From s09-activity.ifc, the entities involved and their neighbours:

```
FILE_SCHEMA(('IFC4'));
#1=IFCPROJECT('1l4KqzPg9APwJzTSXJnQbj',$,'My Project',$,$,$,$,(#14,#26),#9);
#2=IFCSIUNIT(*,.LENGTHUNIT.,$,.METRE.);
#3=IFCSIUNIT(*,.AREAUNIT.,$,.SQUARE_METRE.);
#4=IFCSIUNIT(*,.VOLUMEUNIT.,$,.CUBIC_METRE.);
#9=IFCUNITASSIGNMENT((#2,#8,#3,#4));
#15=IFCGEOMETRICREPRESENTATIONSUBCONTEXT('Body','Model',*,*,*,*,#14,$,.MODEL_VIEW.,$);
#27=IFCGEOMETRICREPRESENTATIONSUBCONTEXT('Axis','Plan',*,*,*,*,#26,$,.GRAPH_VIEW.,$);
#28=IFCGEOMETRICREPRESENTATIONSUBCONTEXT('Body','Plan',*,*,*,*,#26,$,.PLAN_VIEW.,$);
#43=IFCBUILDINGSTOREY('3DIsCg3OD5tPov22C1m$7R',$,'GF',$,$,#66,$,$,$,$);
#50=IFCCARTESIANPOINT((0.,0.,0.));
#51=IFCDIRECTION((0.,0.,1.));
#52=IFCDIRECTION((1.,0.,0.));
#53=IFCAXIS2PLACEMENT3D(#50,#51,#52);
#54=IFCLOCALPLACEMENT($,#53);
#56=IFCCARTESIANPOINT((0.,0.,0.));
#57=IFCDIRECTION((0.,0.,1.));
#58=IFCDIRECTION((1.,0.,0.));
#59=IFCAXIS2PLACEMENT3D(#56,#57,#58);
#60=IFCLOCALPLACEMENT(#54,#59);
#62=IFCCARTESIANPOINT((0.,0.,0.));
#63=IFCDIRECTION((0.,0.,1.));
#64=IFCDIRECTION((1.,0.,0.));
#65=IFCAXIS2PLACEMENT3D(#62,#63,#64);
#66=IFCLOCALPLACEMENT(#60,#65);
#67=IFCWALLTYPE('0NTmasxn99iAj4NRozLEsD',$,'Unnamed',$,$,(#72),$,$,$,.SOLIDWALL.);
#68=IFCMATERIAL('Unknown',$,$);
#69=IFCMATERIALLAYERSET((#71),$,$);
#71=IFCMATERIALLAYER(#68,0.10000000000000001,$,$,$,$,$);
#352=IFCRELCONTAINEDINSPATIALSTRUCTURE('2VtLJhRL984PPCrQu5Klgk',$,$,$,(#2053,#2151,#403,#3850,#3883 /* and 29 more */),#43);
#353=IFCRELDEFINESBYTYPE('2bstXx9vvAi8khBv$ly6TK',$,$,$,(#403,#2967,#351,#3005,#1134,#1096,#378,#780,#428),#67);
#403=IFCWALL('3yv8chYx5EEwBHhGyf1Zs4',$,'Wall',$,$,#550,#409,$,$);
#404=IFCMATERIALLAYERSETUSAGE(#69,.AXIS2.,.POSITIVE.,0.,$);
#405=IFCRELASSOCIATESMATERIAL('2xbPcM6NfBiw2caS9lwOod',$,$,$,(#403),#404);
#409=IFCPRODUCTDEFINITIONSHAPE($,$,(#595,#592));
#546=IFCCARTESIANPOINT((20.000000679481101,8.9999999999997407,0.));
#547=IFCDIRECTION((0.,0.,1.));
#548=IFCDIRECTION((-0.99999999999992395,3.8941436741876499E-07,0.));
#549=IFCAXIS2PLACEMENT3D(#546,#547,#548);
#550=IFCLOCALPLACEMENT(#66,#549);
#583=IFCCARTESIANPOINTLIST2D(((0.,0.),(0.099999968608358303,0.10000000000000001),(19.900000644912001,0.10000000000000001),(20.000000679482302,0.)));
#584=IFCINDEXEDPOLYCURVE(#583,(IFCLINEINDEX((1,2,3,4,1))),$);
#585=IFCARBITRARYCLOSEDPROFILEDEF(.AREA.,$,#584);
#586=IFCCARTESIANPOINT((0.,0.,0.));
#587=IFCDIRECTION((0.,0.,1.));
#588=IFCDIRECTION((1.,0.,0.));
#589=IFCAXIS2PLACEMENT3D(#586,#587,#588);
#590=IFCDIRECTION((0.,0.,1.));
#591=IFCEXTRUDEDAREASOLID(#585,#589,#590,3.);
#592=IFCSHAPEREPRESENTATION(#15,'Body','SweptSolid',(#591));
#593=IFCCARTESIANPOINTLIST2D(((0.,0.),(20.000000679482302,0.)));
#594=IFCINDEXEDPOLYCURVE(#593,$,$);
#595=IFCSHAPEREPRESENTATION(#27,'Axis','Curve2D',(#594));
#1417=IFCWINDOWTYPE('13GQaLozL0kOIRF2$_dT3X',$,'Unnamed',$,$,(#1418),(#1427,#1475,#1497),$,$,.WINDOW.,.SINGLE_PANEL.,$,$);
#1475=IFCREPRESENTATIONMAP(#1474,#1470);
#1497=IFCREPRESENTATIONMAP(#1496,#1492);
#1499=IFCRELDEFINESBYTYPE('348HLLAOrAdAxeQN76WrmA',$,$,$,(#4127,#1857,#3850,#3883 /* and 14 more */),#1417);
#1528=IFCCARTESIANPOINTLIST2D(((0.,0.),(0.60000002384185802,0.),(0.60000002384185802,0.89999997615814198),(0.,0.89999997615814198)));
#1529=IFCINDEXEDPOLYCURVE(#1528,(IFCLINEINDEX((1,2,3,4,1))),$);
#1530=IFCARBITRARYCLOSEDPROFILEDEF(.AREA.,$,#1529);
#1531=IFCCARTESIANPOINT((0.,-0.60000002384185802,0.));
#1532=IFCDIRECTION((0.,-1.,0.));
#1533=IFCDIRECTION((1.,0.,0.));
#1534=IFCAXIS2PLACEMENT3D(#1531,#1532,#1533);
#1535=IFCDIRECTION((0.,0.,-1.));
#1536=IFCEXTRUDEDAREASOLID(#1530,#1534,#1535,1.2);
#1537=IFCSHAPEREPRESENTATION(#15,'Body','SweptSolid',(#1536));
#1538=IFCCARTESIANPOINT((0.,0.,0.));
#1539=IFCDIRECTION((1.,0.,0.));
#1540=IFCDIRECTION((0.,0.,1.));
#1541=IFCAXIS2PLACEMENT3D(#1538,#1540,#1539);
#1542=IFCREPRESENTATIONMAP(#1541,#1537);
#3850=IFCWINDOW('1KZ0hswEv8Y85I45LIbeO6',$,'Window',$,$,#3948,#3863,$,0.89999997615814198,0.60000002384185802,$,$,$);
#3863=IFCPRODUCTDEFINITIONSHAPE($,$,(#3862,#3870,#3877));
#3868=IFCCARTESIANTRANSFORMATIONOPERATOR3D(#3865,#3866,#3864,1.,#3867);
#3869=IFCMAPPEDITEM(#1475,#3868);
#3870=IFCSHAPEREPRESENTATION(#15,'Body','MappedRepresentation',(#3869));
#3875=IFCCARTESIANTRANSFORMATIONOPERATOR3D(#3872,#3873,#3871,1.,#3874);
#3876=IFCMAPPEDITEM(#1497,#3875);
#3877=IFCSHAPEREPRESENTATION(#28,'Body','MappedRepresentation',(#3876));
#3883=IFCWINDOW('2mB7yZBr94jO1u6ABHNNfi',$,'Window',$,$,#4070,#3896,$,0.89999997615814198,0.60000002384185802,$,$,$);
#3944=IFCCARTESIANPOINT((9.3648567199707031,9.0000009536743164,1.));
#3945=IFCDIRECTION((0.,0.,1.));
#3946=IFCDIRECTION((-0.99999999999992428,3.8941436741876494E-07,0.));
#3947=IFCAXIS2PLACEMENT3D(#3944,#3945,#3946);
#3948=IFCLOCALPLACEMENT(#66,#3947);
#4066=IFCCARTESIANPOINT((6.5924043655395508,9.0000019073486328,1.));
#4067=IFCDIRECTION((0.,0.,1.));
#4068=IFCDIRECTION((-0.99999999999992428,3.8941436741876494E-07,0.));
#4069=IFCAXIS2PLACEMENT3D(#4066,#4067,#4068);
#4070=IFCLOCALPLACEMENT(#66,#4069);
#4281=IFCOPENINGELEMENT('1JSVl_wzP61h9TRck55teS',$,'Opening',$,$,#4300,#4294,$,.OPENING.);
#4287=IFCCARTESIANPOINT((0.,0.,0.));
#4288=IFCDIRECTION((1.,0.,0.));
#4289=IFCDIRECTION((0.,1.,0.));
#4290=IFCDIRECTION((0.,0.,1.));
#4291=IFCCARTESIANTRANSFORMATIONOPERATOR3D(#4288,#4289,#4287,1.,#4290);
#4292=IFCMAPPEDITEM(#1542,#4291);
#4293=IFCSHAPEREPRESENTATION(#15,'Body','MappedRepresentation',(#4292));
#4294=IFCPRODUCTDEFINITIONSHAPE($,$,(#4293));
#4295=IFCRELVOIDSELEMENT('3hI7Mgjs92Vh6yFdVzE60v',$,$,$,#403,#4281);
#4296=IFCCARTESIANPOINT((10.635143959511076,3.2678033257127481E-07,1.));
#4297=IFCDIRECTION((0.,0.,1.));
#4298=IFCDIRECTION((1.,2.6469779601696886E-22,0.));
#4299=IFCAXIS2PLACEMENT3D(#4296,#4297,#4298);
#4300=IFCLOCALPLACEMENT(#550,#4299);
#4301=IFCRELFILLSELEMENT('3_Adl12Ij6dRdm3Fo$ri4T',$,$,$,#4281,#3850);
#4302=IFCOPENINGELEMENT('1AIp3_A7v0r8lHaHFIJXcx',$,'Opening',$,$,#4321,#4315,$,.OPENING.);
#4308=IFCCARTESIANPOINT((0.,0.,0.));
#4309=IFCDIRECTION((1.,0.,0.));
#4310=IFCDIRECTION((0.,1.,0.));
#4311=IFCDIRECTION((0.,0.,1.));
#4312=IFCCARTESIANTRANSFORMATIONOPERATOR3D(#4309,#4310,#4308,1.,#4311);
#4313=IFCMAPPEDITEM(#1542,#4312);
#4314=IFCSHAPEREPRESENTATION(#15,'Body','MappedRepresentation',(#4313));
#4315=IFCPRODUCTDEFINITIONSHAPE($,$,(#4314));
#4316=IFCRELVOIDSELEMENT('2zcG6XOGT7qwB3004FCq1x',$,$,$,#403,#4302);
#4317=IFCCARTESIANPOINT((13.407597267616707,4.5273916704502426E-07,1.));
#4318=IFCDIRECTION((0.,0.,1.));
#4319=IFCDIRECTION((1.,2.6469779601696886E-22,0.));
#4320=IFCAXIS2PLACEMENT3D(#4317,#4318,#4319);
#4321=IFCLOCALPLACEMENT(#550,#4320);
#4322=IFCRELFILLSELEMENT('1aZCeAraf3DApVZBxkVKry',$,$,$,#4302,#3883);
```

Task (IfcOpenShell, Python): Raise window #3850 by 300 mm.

```python
import numpy as np
import ifcopenshell
import ifcopenshell.api.geometry
import ifcopenshell.util.placement
import ifcopenshell.util.unit

model = ifcopenshell.open("s09-activity.ifc")
unit_scale = ifcopenshell.util.unit.calculate_unit_scale(model)

window = model.by_id(3850)
opening = window.FillsVoids[0].RelatingOpeningElement
dz = 0.3

shift = np.array([0.0, 0.0, dz])
# The window is not placed relative to its opening, so move both.
for product in (opening, window):
    matrix = ifcopenshell.util.placement.get_local_placement(product.ObjectPlacement)
    matrix[:3, 3] += shift
    ifcopenshell.api.geometry.edit_object_placement(model, product=product, matrix=matrix, is_si=False)

print(f"moved by {dz * unit_scale:+.3f} m")

model.write("s09-activity_rev.ifc")
```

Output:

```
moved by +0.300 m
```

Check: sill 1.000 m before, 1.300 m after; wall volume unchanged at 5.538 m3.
